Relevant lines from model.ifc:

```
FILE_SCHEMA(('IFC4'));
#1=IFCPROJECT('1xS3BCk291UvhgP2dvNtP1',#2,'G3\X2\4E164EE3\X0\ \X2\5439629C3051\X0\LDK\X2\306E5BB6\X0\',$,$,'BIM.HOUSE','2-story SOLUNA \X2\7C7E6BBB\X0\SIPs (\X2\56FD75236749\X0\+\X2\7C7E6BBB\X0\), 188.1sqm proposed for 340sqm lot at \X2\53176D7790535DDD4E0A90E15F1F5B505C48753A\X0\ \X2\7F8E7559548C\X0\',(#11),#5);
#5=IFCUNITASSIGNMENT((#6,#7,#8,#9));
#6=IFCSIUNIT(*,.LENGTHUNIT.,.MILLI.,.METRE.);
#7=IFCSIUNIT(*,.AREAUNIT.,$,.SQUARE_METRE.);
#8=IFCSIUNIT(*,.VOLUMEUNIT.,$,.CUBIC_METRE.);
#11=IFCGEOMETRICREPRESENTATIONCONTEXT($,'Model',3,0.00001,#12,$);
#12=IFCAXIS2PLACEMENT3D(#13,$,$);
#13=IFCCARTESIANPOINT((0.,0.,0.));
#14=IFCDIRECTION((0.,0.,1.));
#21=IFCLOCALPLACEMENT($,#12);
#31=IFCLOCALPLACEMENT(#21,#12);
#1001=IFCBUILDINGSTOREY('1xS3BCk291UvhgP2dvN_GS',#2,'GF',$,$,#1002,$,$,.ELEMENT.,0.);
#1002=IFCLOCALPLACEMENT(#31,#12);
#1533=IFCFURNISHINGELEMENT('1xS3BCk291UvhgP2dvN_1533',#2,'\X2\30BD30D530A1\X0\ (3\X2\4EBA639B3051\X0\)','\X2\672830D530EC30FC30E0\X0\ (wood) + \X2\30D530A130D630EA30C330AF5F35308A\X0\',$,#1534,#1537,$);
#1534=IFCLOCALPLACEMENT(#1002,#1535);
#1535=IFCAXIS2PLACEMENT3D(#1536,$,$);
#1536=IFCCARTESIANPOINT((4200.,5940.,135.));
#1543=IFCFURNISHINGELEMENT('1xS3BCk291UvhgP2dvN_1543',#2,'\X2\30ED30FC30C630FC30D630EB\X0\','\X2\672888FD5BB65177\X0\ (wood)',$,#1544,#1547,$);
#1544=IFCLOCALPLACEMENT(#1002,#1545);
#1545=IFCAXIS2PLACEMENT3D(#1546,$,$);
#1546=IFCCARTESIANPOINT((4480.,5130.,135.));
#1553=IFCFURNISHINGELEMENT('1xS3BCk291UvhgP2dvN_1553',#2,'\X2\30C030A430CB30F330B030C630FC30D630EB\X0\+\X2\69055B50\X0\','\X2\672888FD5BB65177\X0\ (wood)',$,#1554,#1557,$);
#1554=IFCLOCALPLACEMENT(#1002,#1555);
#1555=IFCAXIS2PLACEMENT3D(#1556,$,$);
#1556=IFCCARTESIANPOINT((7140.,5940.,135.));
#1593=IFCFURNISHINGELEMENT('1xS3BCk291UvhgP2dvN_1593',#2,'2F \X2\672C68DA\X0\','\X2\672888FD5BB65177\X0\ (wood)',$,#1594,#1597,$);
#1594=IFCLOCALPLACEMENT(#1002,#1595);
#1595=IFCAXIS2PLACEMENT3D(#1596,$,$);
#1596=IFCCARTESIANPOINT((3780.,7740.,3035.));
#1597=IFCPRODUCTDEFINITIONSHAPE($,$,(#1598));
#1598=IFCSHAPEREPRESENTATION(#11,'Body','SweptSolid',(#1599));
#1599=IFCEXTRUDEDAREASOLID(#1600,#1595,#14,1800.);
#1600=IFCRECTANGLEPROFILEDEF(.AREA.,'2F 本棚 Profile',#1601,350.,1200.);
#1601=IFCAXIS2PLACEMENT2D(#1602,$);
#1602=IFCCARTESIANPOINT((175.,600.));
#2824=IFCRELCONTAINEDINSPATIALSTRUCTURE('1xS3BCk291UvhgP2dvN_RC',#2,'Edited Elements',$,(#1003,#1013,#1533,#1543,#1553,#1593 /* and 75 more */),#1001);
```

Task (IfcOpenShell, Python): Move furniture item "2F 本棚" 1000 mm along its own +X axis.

```python
import ifcopenshell
import ifcopenshell.api.geometry
import ifcopenshell.util.placement

model = ifcopenshell.open("model.ifc")

item = model.by_guid("1xS3BCk291UvhgP2dvN_1593")
matrix = ifcopenshell.util.placement.get_local_placement(item.ObjectPlacement)
matrix[:3, 3] += matrix[:3, 0] * 1000.0
ifcopenshell.api.geometry.edit_object_placement(model, product=item, matrix=matrix, is_si=False)

print(ifcopenshell.util.placement.get_local_placement(item.ObjectPlacement).round(3) + 0.0)

model.write("model_v2.ifc")
```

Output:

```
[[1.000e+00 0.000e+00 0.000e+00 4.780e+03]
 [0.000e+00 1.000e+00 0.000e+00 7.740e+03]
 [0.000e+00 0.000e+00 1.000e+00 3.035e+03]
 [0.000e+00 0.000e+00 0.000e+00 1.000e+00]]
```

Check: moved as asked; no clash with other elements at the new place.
